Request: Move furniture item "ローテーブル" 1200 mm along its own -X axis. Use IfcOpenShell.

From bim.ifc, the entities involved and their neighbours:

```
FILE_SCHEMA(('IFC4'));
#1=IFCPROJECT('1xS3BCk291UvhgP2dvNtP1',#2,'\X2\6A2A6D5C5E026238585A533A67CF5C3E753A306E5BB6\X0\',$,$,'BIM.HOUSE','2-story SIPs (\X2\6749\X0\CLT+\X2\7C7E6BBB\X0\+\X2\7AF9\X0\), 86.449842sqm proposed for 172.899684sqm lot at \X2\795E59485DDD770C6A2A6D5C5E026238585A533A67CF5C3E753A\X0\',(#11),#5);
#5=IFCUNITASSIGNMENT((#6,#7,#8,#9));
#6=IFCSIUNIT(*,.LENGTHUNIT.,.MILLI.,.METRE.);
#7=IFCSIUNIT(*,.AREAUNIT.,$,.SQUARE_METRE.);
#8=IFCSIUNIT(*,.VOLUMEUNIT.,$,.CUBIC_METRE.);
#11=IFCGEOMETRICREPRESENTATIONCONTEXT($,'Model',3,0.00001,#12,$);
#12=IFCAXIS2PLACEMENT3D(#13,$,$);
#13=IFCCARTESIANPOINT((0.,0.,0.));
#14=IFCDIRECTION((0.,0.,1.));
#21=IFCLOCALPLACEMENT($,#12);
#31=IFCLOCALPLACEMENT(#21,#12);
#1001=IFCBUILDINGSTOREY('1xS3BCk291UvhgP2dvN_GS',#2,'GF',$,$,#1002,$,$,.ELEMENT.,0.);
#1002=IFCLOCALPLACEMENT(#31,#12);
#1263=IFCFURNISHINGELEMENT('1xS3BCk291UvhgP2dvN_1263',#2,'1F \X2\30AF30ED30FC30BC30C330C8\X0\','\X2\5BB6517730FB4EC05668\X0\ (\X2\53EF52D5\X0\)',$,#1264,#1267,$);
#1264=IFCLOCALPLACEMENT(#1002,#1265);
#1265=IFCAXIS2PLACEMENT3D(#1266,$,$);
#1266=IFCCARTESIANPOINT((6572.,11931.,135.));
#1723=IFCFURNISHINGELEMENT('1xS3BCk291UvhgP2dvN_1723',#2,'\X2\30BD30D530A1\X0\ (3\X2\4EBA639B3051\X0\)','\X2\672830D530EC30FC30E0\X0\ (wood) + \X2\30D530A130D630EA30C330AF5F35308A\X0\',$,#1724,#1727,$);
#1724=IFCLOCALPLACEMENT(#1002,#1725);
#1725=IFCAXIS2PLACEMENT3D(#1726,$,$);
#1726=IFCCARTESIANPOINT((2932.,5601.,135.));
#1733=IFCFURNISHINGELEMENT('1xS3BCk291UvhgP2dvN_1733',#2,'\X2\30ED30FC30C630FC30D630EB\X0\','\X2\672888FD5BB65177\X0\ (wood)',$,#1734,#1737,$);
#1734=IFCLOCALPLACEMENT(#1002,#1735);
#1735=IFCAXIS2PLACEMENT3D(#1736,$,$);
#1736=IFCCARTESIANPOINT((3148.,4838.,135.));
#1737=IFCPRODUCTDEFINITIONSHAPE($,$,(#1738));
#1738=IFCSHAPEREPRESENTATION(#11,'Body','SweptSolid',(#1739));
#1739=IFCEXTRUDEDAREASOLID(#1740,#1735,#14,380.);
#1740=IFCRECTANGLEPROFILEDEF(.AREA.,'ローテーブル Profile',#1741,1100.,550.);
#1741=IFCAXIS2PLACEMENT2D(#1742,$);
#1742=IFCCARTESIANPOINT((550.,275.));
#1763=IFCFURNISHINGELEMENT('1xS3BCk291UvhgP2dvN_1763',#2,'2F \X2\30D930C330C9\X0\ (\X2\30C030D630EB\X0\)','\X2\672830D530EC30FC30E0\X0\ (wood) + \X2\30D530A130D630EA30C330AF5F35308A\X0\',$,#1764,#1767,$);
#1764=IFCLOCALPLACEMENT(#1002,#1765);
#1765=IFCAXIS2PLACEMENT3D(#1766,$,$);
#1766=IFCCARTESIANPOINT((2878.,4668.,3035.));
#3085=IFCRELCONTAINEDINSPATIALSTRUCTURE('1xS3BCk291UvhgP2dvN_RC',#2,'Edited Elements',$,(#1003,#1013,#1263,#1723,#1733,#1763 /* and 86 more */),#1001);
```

```python
import ifcopenshell
import ifcopenshell.api.geometry
import ifcopenshell.util.placement
import ifcopenshell.util.unit

model = ifcopenshell.open("bim.ifc")
unit_scale = ifcopenshell.util.unit.calculate_unit_scale(model)

item = model.by_guid("1xS3BCk291UvhgP2dvN_1733")
matrix = ifcopenshell.util.placement.get_local_placement(item.ObjectPlacement)
matrix[:3, 3] -= matrix[:3, 0] * 1.2 / unit_scale
ifcopenshell.api.geometry.edit_object_placement(model, product=item, matrix=matrix, is_si=False)

print(ifcopenshell.util.placement.get_local_placement(item.ObjectPlacement).round(3) + 0.0)

model.write("bim_edited.ifc")
```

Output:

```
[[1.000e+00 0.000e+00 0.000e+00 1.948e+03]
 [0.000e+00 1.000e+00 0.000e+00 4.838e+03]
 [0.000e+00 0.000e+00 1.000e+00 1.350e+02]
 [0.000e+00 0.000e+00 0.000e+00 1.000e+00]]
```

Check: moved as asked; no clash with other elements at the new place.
